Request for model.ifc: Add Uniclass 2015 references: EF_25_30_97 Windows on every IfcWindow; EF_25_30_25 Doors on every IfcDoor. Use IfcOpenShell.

First a look at what the model holds.

```python
import ifcopenshell

model = ifcopenshell.open("model.ifc")
print(model.schema)
print("classifications:", [c.Name for c in model.by_type("IfcClassification")])
for ifc_class in ("IfcDoor", "IfcRoof", "IfcStair", "IfcWall", "IfcWindow"):
    print(ifc_class, len(model.by_type(ifc_class)))
```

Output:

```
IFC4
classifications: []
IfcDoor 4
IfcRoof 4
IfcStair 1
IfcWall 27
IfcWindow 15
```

```python
import ifcopenshell
import ifcopenshell.api.classification

model = ifcopenshell.open("model.ifc")

system = ifcopenshell.api.classification.add_classification(model, classification="Uniclass 2015")

codes = {
    "IfcWindow": ("EF_25_30_97", "Windows"),
    "IfcDoor": ("EF_25_30_25", "Doors"),
}
for ifc_class, (code, name) in codes.items():
    products = model.by_type(ifc_class)
    ifcopenshell.api.classification.add_reference(
        model, products=products, classification=system, identification=code, name=name
    )
    print(code, len(products))

model.write("model-out.ifc")
```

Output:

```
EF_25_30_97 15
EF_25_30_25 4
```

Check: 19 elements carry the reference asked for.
